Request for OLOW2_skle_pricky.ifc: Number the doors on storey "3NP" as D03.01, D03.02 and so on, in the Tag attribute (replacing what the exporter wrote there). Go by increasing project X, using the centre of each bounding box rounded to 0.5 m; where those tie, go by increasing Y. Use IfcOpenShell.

First a look at what the model holds.

```python
import ifcopenshell
import ifcopenshell.util.element
import ifcopenshell.util.placement

model = ifcopenshell.open("OLOW2_skle_pricky.ifc")
print(model.schema)
storey = next(s for s in model.by_type("IfcBuildingStorey") if s.Name == "3NP")
doors = [e for e in ifcopenshell.util.element.get_decomposition(storey) if e.is_a("IfcDoor")]
for e in sorted(doors, key=lambda e: e.id()):
    origin = ifcopenshell.util.placement.get_local_placement(e.ObjectPlacement)[:3, 3]
    print(e.id(), e.Tag, e.Name, origin.round(2) + 0.0, sep=" | ")
```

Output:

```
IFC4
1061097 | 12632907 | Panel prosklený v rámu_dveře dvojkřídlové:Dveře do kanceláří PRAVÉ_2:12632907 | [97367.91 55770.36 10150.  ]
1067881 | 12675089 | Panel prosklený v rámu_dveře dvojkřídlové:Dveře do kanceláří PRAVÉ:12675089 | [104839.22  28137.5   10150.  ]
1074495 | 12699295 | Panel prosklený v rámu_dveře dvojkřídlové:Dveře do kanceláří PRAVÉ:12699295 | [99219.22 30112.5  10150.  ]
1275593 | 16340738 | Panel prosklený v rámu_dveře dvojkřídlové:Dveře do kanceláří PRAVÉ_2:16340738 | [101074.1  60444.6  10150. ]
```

```python
import ifcopenshell
import ifcopenshell.geom
import ifcopenshell.util.element
import ifcopenshell.util.shape

model = ifcopenshell.open("OLOW2_skle_pricky.ifc")
settings = ifcopenshell.geom.settings()
settings.set("use-world-coords", True)


def centre(element):
    shape = ifcopenshell.geom.create_shape(settings, element)
    return ifcopenshell.util.shape.get_bbox_centroid(shape.geometry)


storey = next(s for s in model.by_type("IfcBuildingStorey") if s.Name == "3NP")
doors = [e for e in ifcopenshell.util.element.get_decomposition(storey) if e.is_a("IfcDoor")]

# Insertion points can sit at a corner or the storey origin, so sort by the geometry (in metres).
centres = {e: centre(e) for e in doors}
doors.sort(key=lambda e: (round(centres[e][0] / 0.5), centres[e][1]))

for i, e in enumerate(doors, start=1):
    number = f"D03.{i:02d}"
    e.Tag = number
    print(e.id(), number)

model.write("OLOW2_skle_pricky-out.ifc")
```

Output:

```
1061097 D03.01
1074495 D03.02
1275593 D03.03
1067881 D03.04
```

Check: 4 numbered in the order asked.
